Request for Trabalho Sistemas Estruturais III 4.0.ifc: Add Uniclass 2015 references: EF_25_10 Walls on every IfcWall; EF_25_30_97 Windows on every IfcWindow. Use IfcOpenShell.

First a look at what the model holds.

```python
import ifcopenshell

model = ifcopenshell.open("Trabalho Sistemas Estruturais III 4.0.ifc")
print(model.schema)
print("classifications:", [c.Name for c in model.by_type("IfcClassification")])
for ifc_class in ("IfcDoor", "IfcRoof", "IfcStair", "IfcWall", "IfcWindow"):
    print(ifc_class, len(model.by_type(ifc_class)))
```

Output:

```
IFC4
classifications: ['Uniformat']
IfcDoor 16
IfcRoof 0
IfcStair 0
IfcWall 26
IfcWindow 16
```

```python
import ifcopenshell
import ifcopenshell.api.classification

model = ifcopenshell.open("Trabalho Sistemas Estruturais III 4.0.ifc")

system = ifcopenshell.api.classification.add_classification(model, classification="Uniclass 2015")

codes = {
    "IfcWall": ("EF_25_10", "Walls"),
    "IfcWindow": ("EF_25_30_97", "Windows"),
}
for ifc_class, (code, name) in codes.items():
    products = model.by_type(ifc_class)
    ifcopenshell.api.classification.add_reference(
        model, products=products, classification=system, identification=code, name=name
    )
    print(code, len(products))

model.write("Trabalho Sistemas Estruturais III 4.0_edited.ifc")
```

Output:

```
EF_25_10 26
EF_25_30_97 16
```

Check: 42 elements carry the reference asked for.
